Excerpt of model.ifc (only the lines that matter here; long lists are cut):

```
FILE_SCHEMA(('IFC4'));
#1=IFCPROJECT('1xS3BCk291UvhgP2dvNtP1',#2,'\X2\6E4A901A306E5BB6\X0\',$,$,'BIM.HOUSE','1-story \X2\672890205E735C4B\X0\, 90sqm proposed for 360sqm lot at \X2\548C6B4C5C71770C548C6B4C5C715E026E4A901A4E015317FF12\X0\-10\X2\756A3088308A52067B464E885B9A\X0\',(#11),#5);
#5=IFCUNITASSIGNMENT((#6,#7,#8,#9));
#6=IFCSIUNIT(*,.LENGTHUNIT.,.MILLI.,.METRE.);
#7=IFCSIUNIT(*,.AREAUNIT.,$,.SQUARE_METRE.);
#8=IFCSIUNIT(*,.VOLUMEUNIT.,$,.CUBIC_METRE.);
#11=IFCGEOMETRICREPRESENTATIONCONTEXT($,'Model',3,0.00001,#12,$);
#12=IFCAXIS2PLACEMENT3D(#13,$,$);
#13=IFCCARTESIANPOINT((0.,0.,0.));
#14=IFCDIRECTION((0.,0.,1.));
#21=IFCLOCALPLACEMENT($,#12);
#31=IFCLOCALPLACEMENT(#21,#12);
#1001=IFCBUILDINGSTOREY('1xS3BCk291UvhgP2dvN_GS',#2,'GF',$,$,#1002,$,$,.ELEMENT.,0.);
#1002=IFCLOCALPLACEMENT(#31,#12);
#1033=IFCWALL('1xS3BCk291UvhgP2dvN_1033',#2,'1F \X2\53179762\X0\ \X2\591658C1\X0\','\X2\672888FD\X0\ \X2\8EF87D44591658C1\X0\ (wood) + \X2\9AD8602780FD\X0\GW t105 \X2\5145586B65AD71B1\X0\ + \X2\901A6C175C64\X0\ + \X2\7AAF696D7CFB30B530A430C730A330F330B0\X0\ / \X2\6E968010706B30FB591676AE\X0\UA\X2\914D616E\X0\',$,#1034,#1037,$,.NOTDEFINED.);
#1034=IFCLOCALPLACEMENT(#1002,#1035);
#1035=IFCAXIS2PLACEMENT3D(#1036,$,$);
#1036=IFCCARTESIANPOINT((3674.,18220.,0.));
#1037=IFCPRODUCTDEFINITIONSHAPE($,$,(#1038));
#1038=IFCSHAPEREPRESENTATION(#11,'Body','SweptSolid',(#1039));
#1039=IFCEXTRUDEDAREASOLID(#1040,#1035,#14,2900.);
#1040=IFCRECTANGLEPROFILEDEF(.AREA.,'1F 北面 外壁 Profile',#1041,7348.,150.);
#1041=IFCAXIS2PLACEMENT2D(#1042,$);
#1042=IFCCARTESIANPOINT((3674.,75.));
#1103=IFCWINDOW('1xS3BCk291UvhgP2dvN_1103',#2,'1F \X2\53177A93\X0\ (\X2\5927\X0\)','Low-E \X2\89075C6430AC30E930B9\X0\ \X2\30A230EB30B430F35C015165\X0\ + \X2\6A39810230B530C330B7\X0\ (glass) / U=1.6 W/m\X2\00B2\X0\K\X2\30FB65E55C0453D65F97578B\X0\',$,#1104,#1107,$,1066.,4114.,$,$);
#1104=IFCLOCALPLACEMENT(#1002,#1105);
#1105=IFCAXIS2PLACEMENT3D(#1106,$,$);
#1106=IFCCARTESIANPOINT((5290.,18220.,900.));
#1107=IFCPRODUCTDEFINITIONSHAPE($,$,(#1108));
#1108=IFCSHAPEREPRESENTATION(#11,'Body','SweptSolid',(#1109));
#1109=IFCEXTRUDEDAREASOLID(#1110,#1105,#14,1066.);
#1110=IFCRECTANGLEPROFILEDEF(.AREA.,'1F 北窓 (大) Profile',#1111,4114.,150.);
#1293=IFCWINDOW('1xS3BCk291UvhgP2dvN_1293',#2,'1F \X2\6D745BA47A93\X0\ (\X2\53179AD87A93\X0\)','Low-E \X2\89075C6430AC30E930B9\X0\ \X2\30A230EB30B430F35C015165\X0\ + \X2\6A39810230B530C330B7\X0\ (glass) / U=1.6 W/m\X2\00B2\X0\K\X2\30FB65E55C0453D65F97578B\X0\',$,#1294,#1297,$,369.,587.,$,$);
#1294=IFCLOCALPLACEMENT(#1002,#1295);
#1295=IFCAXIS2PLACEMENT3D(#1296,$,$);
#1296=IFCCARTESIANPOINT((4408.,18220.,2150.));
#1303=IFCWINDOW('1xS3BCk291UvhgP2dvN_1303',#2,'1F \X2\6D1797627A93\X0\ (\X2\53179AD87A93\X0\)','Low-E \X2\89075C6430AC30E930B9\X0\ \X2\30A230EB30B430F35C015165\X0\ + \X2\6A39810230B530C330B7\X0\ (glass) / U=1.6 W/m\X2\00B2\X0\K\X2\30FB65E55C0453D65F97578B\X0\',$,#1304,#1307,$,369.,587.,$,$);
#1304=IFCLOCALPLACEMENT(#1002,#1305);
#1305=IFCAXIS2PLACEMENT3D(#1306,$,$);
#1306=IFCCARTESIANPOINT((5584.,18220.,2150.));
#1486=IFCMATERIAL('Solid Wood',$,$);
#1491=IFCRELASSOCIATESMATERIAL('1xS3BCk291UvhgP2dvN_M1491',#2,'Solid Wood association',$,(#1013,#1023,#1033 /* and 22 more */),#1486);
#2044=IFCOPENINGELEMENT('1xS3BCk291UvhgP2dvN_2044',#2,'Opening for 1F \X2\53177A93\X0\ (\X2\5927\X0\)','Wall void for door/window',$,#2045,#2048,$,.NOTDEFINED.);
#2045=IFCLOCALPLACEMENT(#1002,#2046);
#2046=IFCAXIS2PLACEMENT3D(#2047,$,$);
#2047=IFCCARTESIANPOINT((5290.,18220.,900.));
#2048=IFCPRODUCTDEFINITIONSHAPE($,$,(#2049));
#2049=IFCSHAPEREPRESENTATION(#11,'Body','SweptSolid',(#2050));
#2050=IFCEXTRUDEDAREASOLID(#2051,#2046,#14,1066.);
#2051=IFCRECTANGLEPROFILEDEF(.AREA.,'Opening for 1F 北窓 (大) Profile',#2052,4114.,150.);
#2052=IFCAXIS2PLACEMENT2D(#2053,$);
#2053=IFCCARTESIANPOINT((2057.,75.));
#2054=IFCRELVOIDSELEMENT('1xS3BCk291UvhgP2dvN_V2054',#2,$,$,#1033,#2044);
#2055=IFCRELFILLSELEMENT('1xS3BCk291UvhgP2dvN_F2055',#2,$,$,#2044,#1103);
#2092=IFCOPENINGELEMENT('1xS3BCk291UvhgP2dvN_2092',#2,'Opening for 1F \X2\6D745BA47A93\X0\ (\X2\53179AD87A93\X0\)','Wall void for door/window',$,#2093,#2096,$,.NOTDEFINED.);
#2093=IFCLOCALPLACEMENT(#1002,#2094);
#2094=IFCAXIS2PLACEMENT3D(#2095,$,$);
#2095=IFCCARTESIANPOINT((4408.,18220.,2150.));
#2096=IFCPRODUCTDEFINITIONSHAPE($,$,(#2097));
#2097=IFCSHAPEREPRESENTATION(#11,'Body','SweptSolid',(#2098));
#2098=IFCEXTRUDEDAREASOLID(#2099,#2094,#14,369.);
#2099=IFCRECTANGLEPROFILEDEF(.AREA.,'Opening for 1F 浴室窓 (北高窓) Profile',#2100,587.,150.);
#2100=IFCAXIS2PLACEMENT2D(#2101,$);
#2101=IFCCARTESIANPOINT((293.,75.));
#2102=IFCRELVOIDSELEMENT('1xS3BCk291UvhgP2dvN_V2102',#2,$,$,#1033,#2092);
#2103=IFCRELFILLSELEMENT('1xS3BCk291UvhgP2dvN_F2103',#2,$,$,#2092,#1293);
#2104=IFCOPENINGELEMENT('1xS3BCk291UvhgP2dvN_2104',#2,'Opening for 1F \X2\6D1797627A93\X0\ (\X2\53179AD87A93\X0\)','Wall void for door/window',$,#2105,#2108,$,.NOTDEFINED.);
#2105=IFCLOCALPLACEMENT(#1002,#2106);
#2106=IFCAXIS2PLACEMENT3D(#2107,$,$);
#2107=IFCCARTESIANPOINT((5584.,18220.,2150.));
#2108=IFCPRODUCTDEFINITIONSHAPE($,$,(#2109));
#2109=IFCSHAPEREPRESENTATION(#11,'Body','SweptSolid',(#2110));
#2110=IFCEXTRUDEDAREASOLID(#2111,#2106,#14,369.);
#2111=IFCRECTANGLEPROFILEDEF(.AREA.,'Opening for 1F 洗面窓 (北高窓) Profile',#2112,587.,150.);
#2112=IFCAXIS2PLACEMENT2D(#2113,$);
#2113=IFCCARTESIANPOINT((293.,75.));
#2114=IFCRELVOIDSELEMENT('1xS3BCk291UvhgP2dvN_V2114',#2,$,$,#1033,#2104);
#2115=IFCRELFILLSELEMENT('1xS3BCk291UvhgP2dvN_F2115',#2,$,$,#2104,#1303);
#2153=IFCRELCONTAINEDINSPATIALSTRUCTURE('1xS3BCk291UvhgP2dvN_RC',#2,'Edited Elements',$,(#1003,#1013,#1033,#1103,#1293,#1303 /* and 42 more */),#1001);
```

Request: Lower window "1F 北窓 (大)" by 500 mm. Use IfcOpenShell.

```python
import numpy as np
import ifcopenshell
import ifcopenshell.api.geometry
import ifcopenshell.util.placement
import ifcopenshell.util.unit

model = ifcopenshell.open("model.ifc")
unit_scale = ifcopenshell.util.unit.calculate_unit_scale(model)

window = model.by_guid("1xS3BCk291UvhgP2dvN_1103")
opening = window.FillsVoids[0].RelatingOpeningElement
dz = -0.5 / unit_scale

shift = np.array([0.0, 0.0, dz])
# The window is not placed relative to its opening, so move both.
for product in (opening, window):
    matrix = ifcopenshell.util.placement.get_local_placement(product.ObjectPlacement)
    matrix[:3, 3] += shift
    ifcopenshell.api.geometry.edit_object_placement(model, product=product, matrix=matrix, is_si=False)

print(f"moved by {dz * unit_scale:+.3f} m")

model.write("model_v2.ifc")
```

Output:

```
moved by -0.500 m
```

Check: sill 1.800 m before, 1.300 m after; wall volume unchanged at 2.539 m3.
